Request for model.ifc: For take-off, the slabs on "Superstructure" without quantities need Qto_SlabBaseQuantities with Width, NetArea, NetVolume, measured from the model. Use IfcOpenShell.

First a look at what the model holds.

```python
import ifcopenshell
import ifcopenshell.util.element
import ifcopenshell.util.unit

model = ifcopenshell.open("model.ifc")
print(model.schema)
for unit_type in ("LENGTHUNIT", "AREAUNIT", "VOLUMEUNIT"):
    print(unit_type, ifcopenshell.util.unit.calculate_unit_scale(model, unit_type))
storey = next(s for s in model.by_type("IfcBuildingStorey") if s.Name == "Superstructure")
slabs = [e for e in ifcopenshell.util.element.get_decomposition(storey) if e.is_a("IfcSlab")]
for e in sorted(slabs, key=lambda e: e.id()):
    print(e.id(), e.is_a(), e.Name, list(ifcopenshell.util.element.get_psets(e, qtos_only=True)), sep=" | ")
```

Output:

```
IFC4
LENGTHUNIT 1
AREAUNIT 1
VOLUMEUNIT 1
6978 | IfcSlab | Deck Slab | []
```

```python
import ifcopenshell
import ifcopenshell.api.pset
import ifcopenshell.geom
import ifcopenshell.util.element
import ifcopenshell.util.shape
import ifcopenshell.util.unit

model = ifcopenshell.open("model.ifc")
unit_scale = ifcopenshell.util.unit.calculate_unit_scale(model)
area_scale = ifcopenshell.util.unit.calculate_unit_scale(model, "AREAUNIT")
volume_scale = ifcopenshell.util.unit.calculate_unit_scale(model, "VOLUMEUNIT")
settings = ifcopenshell.geom.settings()

storey = next(s for s in model.by_type("IfcBuildingStorey") if s.Name == "Superstructure")
slabs = [e for e in ifcopenshell.util.element.get_decomposition(storey) if e.is_a("IfcSlab")]

for e in sorted(slabs, key=lambda e: e.id()):
    if ifcopenshell.util.element.get_psets(e, qtos_only=True, should_inherit=False):
        continue
    # Geometry comes back in metres, in the element's own axes.
    shape = ifcopenshell.geom.create_shape(settings, e)
    values = {
        "Width": ifcopenshell.util.shape.get_z(shape.geometry) / unit_scale,
        "NetArea": ifcopenshell.util.shape.get_footprint_area(shape.geometry) / area_scale,
        "NetVolume": ifcopenshell.util.shape.get_volume(shape.geometry) / volume_scale,
    }
    qto = ifcopenshell.api.pset.add_qto(model, product=e, name="Qto_SlabBaseQuantities")
    ifcopenshell.api.pset.edit_qto(model, qto=qto, properties=values)
    print(e.id(), {k: round(v, 3) for k, v in values.items()})

model.write("model_edited.ifc")
```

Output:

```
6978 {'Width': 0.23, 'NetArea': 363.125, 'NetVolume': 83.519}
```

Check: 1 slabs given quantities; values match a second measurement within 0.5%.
